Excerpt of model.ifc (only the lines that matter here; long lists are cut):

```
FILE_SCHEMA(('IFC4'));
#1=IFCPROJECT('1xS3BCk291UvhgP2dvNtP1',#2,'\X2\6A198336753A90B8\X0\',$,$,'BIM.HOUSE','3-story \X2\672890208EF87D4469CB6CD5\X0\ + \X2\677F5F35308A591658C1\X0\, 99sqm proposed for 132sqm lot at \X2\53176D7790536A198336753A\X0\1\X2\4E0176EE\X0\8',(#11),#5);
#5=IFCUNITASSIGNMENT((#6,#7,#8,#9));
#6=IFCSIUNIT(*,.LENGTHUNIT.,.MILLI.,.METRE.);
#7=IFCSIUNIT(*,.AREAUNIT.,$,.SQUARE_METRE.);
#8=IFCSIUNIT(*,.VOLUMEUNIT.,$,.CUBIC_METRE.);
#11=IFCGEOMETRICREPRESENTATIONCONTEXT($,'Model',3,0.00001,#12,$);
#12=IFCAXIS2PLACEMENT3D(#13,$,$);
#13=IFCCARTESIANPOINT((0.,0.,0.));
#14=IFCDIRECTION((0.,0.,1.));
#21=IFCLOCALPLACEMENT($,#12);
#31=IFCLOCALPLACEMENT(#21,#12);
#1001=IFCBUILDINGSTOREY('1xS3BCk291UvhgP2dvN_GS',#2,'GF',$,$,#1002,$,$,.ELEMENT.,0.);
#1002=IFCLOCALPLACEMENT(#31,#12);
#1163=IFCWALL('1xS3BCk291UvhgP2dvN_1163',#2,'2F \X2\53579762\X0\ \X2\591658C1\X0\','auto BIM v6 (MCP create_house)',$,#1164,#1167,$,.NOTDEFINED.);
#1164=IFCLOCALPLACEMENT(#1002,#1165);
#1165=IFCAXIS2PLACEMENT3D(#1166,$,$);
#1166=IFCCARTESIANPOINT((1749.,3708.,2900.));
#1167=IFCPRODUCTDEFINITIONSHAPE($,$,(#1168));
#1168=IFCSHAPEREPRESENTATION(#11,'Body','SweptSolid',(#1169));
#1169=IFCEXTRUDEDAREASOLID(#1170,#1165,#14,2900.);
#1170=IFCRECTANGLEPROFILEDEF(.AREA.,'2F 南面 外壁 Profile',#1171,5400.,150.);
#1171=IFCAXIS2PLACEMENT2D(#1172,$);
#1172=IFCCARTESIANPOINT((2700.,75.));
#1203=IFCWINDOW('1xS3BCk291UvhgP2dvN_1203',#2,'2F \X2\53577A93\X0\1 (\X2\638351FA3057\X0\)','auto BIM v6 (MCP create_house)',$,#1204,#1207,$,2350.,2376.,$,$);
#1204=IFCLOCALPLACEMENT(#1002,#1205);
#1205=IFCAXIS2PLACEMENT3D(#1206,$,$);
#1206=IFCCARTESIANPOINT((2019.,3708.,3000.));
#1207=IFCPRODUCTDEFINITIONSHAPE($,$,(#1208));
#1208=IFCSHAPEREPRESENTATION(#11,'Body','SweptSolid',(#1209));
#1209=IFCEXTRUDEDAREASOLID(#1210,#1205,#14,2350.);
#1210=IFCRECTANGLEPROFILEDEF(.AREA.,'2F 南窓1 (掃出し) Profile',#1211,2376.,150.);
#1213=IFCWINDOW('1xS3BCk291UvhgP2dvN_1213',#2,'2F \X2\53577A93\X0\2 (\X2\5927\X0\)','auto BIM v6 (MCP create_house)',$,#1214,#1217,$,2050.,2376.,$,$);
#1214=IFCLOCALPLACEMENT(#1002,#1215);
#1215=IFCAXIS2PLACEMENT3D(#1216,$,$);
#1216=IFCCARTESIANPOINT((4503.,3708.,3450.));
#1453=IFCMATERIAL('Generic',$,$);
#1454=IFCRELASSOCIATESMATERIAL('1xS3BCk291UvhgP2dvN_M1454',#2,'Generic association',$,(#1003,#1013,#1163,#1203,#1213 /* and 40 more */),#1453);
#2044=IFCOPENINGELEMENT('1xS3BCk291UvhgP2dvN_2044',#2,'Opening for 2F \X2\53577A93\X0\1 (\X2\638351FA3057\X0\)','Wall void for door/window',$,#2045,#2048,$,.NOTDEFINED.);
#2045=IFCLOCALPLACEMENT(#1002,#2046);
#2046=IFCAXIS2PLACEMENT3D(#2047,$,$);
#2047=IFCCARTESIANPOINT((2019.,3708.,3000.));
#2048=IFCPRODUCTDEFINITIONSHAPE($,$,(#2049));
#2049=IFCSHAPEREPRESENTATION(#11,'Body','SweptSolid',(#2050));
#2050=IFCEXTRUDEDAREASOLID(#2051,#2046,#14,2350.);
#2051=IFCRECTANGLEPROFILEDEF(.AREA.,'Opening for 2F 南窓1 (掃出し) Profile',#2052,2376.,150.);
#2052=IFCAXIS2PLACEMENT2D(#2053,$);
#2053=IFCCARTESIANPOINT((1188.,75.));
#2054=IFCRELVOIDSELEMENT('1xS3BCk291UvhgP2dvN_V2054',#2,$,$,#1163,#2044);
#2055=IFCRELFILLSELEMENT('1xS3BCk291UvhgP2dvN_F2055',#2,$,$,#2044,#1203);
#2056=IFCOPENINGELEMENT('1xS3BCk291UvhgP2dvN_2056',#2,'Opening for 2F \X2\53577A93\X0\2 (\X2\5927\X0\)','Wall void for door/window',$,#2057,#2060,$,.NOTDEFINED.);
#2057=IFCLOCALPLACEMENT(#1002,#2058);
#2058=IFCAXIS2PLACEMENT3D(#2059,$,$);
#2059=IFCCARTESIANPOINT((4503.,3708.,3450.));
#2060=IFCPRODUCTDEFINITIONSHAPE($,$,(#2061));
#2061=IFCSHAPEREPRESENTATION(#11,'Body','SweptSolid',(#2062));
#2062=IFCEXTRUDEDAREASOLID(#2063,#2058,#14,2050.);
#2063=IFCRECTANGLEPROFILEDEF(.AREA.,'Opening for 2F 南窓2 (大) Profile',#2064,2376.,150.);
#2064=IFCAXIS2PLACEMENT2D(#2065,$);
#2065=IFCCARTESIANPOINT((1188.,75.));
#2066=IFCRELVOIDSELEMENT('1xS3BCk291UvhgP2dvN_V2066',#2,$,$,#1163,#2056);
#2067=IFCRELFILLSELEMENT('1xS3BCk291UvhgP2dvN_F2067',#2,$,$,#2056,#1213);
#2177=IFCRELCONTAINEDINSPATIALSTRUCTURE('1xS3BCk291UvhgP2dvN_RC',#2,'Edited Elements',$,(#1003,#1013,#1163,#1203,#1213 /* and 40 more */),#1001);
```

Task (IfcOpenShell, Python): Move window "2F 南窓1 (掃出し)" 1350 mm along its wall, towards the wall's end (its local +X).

```python
import ifcopenshell
import ifcopenshell.api.geometry
import ifcopenshell.util.placement
import ifcopenshell.util.unit

model = ifcopenshell.open("model.ifc")
unit_scale = ifcopenshell.util.unit.calculate_unit_scale(model)

window = model.by_id(1203)
opening = window.FillsVoids[0].RelatingOpeningElement
wall = opening.VoidsElements[0].RelatingBuildingElement

wall_matrix = ifcopenshell.util.placement.get_local_placement(wall.ObjectPlacement)
shift = wall_matrix[:3, 0] * 1.35 / unit_scale
before = ifcopenshell.util.placement.get_local_placement(window.ObjectPlacement)[:3, 3].copy()

# The window is not placed relative to its opening, so move both.
for product in (opening, window):
    matrix = ifcopenshell.util.placement.get_local_placement(product.ObjectPlacement)
    matrix[:3, 3] += shift
    ifcopenshell.api.geometry.edit_object_placement(model, product=product, matrix=matrix, is_si=False)

after = ifcopenshell.util.placement.get_local_placement(window.ObjectPlacement)[:3, 3]
print("window moved by", (after - before).round(3) + 0.0)

model.write("model_updated.ifc")
```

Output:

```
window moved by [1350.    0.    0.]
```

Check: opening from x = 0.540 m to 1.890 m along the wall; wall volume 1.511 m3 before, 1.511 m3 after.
